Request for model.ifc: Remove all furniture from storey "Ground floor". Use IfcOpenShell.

First a look at what the model holds.

```python
import ifcopenshell
import ifcopenshell.util.element

model = ifcopenshell.open("model.ifc")
print(model.schema)
storey = next(s for s in model.by_type("IfcBuildingStorey") if s.Name == "Ground floor")
furniture = [e for e in ifcopenshell.util.element.get_decomposition(storey) if e.is_a("IfcFurnishingElement")]
seen = {}
for e in furniture:
    element_type = ifcopenshell.util.element.get_type(e)
    name = element_type.Name if element_type not in (None, e) else None
    seen[name] = seen.get(name, 0) + 1
for name, count in sorted(seen.items(), key=str):
    print(count, "x", name)
```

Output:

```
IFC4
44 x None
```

```python
import ifcopenshell
import ifcopenshell.api.root
import ifcopenshell.util.element

model = ifcopenshell.open("model.ifc")

storey = next(s for s in model.by_type("IfcBuildingStorey") if s.Name == "Ground floor")
furniture = [e for e in ifcopenshell.util.element.get_decomposition(storey) if e.is_a("IfcFurnishingElement")]

for e in furniture:
    ifcopenshell.api.root.remove_product(model, product=e)
print(len(furniture), "removed")

model.write("model_edited.ifc")
```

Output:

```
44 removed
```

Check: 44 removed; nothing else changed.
